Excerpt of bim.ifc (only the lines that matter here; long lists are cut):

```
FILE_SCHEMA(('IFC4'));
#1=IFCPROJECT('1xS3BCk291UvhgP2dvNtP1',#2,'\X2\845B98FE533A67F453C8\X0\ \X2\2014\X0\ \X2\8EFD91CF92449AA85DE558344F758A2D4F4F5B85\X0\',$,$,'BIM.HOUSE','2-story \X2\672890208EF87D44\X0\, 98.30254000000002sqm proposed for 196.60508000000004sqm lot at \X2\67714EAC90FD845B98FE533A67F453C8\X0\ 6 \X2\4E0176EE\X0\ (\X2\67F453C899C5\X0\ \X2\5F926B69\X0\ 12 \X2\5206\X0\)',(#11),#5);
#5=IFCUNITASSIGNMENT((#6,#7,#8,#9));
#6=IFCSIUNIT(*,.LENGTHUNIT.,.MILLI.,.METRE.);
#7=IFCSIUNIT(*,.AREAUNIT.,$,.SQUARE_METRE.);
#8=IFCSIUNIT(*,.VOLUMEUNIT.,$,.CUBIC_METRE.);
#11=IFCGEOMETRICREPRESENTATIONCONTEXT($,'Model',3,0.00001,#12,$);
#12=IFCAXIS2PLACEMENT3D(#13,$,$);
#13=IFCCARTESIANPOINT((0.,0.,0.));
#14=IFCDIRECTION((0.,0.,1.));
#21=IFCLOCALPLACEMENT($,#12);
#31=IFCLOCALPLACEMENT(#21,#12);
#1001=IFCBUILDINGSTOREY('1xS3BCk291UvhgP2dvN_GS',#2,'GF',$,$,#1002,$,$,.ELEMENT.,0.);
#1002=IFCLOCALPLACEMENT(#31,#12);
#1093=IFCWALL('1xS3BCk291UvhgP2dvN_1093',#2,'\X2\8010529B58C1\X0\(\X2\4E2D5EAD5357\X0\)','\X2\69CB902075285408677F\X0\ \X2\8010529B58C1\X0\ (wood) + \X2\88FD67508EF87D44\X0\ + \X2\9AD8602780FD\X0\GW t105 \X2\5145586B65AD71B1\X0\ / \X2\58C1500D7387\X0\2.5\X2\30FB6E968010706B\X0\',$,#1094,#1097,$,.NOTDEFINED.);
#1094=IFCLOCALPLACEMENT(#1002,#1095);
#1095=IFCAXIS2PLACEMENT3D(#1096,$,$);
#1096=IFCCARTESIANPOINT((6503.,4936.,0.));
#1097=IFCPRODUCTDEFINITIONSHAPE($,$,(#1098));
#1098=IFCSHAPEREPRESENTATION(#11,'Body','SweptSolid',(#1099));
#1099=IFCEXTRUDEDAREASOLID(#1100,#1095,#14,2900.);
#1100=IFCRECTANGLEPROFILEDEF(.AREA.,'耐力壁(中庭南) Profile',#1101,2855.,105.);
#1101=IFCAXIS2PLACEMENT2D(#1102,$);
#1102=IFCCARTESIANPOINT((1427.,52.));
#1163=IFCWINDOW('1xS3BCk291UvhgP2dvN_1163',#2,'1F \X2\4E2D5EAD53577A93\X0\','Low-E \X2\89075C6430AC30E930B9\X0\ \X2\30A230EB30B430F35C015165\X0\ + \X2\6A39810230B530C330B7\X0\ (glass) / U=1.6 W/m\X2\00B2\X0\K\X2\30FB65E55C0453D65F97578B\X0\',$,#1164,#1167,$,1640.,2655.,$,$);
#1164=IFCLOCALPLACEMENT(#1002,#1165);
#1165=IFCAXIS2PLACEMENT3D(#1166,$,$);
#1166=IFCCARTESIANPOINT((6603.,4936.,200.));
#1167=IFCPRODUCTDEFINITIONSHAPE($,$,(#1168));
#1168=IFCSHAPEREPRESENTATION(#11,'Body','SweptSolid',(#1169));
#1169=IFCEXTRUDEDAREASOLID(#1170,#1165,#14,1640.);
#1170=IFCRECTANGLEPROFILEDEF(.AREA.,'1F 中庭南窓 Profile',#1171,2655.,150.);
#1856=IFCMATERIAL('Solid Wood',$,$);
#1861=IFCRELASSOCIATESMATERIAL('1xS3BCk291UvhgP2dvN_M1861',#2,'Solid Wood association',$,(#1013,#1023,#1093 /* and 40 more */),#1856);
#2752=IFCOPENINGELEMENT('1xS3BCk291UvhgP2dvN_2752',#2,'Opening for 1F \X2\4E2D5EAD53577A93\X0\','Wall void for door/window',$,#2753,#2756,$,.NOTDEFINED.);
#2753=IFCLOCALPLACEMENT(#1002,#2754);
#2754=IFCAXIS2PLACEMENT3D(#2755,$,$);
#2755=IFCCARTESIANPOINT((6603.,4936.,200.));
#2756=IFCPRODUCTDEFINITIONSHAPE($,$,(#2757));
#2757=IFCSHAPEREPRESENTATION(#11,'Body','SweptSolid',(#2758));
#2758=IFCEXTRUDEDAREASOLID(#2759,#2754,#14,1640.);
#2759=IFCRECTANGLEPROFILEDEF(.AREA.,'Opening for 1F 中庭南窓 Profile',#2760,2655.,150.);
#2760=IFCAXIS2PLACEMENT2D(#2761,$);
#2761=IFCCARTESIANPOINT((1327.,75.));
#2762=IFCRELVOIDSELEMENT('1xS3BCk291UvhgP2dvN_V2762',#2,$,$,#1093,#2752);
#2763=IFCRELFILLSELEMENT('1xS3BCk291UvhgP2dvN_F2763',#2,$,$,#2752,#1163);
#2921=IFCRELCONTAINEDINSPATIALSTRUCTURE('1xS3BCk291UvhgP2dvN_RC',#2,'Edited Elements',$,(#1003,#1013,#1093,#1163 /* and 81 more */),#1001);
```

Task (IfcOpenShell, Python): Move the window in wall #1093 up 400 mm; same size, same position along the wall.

```python
import numpy as np
import ifcopenshell
import ifcopenshell.api.geometry
import ifcopenshell.util.placement
import ifcopenshell.util.unit

model = ifcopenshell.open("bim.ifc")
unit_scale = ifcopenshell.util.unit.calculate_unit_scale(model)

window = model.by_id(1163)
opening = window.FillsVoids[0].RelatingOpeningElement
dz = 0.4 / unit_scale

shift = np.array([0.0, 0.0, dz])
# The window is not placed relative to its opening, so move both.
for product in (opening, window):
    matrix = ifcopenshell.util.placement.get_local_placement(product.ObjectPlacement)
    matrix[:3, 3] += shift
    ifcopenshell.api.geometry.edit_object_placement(model, product=product, matrix=matrix, is_si=False)

print(f"moved by {dz * unit_scale:+.3f} m")

model.write("bim_v2.ifc")
```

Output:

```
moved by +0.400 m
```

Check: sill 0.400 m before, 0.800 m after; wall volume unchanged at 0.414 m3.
